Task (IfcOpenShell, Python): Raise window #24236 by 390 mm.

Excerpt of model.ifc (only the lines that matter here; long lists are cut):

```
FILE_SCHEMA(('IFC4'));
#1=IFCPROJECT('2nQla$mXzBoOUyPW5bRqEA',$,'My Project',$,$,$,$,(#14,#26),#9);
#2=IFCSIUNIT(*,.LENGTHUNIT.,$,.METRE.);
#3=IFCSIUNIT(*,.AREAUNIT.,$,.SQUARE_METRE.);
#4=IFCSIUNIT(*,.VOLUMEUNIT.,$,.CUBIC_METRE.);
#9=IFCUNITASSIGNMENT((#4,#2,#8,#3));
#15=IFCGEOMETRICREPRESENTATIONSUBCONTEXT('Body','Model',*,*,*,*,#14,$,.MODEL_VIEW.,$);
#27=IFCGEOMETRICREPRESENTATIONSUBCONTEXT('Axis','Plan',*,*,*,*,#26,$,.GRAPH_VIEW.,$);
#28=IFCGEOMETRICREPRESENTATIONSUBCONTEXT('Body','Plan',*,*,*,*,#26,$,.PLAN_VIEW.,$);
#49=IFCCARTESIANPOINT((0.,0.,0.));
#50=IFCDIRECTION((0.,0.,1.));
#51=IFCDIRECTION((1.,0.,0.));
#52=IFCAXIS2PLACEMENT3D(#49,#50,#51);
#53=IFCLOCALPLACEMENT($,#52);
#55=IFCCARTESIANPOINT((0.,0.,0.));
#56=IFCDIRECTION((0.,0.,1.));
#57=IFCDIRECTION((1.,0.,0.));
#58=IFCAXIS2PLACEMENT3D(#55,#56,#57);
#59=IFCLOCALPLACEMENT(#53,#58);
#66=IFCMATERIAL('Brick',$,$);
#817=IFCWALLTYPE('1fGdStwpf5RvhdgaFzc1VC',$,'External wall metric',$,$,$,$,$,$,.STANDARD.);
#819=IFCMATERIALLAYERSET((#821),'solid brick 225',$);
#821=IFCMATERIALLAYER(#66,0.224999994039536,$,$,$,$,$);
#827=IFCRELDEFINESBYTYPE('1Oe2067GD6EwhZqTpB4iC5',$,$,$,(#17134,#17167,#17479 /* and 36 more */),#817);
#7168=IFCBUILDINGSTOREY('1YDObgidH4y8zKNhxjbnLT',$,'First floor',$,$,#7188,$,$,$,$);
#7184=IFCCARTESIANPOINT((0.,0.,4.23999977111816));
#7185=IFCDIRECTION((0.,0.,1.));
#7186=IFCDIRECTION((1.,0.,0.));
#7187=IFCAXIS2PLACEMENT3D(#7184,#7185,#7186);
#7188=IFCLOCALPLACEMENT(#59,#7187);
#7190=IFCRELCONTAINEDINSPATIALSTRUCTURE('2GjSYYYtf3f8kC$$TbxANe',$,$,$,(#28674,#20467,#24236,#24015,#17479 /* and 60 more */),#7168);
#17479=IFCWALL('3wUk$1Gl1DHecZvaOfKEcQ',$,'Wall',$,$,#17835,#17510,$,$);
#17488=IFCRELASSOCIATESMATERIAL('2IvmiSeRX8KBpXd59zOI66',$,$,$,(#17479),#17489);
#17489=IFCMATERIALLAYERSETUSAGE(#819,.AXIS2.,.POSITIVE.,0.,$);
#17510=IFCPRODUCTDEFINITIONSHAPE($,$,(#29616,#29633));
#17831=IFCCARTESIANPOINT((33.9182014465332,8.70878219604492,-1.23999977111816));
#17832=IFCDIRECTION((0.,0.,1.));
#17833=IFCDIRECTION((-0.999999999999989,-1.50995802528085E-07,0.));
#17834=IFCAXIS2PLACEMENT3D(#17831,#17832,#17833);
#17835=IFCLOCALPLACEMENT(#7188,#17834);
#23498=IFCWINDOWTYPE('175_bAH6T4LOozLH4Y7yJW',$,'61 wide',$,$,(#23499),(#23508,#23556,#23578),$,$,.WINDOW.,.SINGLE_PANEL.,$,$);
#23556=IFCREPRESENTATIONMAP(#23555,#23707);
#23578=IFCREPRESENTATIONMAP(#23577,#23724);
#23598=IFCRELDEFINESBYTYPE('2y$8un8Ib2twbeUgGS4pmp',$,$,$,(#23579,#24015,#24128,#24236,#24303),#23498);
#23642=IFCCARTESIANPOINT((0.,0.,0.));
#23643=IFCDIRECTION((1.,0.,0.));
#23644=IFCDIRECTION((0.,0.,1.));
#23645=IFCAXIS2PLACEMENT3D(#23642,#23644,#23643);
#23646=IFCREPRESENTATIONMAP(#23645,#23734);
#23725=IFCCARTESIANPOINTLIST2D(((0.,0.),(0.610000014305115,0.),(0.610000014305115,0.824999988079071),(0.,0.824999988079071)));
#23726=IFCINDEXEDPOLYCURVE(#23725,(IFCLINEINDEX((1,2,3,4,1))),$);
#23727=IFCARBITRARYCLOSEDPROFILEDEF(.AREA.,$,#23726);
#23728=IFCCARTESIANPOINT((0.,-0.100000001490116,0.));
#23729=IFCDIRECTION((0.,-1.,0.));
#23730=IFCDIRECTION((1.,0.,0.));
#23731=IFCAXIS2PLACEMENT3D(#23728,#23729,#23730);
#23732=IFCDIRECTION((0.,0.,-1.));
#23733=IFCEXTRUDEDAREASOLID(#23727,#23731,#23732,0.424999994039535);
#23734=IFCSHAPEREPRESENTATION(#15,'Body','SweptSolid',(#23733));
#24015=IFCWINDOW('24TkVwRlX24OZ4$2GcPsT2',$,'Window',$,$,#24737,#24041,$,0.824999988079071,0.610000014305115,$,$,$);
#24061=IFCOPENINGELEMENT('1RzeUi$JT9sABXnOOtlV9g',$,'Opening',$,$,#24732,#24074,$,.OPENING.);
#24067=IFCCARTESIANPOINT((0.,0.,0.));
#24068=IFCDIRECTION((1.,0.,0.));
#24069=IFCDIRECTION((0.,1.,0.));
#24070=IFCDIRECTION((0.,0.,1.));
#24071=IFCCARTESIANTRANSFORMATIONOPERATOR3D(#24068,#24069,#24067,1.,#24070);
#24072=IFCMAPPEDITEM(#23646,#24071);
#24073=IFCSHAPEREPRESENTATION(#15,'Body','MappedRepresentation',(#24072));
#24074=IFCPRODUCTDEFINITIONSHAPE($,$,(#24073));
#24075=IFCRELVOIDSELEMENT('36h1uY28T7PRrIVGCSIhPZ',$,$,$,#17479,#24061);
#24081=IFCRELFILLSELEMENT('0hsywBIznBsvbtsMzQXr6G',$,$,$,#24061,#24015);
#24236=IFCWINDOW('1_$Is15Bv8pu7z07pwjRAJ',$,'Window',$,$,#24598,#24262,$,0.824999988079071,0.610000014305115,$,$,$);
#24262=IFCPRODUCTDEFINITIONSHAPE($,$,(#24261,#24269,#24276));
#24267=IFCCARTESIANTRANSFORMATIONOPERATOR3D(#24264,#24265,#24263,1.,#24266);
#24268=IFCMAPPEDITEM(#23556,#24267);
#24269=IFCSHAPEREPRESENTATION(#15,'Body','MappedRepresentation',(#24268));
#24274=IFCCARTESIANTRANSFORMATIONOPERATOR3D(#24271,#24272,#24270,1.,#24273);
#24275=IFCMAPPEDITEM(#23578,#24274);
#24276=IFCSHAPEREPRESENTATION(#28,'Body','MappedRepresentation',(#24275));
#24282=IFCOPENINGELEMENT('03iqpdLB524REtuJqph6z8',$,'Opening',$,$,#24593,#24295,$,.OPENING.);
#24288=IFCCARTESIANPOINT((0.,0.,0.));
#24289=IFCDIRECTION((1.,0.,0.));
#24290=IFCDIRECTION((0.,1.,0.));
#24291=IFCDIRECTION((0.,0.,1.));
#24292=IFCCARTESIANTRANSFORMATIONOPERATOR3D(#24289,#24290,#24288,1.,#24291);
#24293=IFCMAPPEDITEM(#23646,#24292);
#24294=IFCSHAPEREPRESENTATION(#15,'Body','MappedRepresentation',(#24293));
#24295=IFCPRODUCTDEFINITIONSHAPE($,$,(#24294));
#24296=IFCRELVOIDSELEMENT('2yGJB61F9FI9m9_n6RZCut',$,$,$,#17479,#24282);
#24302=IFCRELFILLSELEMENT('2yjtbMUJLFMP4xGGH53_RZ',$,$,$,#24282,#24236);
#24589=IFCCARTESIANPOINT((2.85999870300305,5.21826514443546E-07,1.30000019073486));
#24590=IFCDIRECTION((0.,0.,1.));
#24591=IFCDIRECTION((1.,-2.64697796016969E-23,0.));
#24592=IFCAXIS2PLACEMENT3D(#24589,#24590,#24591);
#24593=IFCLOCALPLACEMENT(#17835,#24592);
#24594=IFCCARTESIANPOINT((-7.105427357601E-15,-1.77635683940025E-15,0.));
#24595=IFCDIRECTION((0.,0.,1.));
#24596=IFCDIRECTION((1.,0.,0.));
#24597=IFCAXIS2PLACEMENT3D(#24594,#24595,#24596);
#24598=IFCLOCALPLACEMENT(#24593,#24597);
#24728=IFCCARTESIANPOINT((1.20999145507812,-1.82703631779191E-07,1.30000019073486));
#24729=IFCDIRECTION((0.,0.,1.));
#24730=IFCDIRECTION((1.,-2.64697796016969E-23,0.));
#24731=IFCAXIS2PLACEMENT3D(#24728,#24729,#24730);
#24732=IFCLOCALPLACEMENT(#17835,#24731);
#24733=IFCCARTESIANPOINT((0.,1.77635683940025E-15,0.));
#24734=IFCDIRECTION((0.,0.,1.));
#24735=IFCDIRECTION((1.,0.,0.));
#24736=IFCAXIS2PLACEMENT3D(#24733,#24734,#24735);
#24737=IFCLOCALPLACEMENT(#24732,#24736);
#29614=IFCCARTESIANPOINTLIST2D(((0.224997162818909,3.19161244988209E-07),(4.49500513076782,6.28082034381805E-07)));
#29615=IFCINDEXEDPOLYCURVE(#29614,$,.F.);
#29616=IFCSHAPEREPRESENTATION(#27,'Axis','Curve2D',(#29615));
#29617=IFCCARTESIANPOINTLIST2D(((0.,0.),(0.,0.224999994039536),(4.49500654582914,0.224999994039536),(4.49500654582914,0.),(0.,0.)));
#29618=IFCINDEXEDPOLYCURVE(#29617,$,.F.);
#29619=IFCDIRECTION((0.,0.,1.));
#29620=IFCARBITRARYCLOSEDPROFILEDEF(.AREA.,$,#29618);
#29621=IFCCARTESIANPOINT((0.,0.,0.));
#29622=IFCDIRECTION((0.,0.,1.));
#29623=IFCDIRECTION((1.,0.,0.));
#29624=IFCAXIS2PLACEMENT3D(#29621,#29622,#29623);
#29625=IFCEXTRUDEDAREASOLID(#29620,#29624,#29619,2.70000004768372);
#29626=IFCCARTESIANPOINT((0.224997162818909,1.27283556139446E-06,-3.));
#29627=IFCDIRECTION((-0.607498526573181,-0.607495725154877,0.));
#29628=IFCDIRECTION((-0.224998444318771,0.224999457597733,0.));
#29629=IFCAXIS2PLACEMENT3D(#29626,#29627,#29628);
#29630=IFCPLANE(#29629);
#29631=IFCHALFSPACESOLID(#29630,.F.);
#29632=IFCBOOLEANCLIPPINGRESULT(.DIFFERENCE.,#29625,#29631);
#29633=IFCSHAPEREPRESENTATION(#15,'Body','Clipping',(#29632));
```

```python
import numpy as np
import ifcopenshell
import ifcopenshell.api.geometry
import ifcopenshell.util.placement
import ifcopenshell.util.unit

model = ifcopenshell.open("model.ifc")
unit_scale = ifcopenshell.util.unit.calculate_unit_scale(model)

window = model.by_id(24236)
opening = window.FillsVoids[0].RelatingOpeningElement
dz = 0.39

shift = np.array([0.0, 0.0, dz])
# The window is placed relative to its opening, so it follows when the opening moves.
matrix = ifcopenshell.util.placement.get_local_placement(opening.ObjectPlacement)
matrix[:3, 3] += shift
ifcopenshell.api.geometry.edit_object_placement(
    model, product=opening, matrix=matrix, is_si=False, should_transform_children=True
)

print(f"moved by {dz * unit_scale:+.3f} m")

model.write("model_rev.ifc")
```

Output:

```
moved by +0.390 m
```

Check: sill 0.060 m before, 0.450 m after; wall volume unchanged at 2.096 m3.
